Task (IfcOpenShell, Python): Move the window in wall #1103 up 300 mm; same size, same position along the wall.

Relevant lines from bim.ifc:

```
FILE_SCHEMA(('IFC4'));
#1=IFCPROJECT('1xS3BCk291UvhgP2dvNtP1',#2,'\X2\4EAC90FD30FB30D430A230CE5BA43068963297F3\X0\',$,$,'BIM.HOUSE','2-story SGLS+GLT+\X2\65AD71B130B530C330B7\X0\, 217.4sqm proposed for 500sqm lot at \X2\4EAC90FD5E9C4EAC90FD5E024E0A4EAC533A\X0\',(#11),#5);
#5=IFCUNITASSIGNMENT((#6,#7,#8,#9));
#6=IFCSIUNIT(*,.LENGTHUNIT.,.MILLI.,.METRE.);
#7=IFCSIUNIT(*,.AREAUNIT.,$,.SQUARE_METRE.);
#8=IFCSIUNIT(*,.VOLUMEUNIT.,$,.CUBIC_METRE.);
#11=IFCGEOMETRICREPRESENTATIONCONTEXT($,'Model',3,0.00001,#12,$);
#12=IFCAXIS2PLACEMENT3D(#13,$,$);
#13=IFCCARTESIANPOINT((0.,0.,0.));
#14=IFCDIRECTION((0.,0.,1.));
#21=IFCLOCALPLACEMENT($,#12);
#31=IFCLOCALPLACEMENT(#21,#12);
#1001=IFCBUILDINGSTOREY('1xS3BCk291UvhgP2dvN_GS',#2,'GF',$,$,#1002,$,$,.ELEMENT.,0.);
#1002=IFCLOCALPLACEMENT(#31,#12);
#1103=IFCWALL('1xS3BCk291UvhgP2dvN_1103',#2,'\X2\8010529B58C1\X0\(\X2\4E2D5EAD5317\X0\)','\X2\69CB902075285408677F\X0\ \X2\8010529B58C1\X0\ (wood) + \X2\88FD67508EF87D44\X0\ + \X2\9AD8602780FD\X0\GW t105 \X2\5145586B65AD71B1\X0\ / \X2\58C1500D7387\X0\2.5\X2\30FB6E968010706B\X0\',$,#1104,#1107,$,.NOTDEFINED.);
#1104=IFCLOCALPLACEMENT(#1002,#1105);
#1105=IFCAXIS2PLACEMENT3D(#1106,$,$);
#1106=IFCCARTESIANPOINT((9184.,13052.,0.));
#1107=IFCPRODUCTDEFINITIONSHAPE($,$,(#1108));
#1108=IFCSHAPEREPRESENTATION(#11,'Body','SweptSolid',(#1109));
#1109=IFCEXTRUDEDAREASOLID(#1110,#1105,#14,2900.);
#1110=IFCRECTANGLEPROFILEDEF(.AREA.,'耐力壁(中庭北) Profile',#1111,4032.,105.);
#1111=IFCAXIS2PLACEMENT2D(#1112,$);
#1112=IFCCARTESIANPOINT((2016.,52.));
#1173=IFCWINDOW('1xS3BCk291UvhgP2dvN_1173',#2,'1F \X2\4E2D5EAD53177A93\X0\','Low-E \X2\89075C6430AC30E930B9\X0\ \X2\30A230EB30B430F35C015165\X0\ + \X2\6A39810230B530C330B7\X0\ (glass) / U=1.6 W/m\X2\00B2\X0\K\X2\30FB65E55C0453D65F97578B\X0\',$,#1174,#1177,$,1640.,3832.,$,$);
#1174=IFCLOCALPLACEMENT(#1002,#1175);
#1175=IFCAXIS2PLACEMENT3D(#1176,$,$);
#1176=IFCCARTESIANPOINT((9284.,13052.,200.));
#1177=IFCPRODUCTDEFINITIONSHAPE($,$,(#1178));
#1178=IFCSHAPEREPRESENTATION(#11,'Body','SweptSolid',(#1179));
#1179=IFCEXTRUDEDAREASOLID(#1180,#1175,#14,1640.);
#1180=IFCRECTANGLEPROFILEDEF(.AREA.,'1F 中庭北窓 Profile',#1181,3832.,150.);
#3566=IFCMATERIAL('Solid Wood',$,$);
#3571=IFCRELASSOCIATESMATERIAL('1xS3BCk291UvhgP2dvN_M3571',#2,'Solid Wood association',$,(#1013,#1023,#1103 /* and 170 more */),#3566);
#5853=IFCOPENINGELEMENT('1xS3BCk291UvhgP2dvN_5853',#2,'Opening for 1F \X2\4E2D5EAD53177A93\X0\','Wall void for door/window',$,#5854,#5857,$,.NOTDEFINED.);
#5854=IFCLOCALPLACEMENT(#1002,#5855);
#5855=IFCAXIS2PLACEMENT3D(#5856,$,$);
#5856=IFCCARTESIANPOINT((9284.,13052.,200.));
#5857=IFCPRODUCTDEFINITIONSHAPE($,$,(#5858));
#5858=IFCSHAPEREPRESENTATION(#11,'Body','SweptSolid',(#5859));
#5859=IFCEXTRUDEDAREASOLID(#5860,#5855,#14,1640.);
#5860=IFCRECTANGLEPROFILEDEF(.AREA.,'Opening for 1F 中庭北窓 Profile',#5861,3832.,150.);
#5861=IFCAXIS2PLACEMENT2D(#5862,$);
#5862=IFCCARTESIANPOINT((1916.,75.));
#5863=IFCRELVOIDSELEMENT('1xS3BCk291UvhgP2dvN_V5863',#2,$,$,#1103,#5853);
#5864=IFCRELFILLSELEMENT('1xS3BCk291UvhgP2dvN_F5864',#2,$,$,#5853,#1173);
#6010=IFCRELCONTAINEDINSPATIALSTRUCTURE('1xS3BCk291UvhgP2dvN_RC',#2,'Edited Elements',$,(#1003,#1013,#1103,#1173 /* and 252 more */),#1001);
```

```python
import numpy as np
import ifcopenshell
import ifcopenshell.api.geometry
import ifcopenshell.util.placement
import ifcopenshell.util.unit

model = ifcopenshell.open("bim.ifc")
unit_scale = ifcopenshell.util.unit.calculate_unit_scale(model)

window = model.by_guid("1xS3BCk291UvhgP2dvN_1173")
opening = window.FillsVoids[0].RelatingOpeningElement
dz = 0.3 / unit_scale

shift = np.array([0.0, 0.0, dz])
# The window is not placed relative to its opening, so move both.
for product in (opening, window):
    matrix = ifcopenshell.util.placement.get_local_placement(product.ObjectPlacement)
    matrix[:3, 3] += shift
    ifcopenshell.api.geometry.edit_object_placement(model, product=product, matrix=matrix, is_si=False)

print(f"moved by {dz * unit_scale:+.3f} m")

model.write("bim-out.ifc")
```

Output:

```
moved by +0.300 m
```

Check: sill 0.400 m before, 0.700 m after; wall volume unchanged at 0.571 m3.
